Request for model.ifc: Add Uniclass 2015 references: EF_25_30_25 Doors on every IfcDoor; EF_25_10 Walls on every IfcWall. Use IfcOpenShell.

First a look at what the model holds.

```python
import ifcopenshell

model = ifcopenshell.open("model.ifc")
print(model.schema)
print("classifications:", [c.Name for c in model.by_type("IfcClassification")])
for ifc_class in ("IfcDoor", "IfcRoof", "IfcStair", "IfcWall", "IfcWindow"):
    print(ifc_class, len(model.by_type(ifc_class)))
```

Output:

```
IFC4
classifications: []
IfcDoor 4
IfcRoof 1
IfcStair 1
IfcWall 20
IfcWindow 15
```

```python
import ifcopenshell
import ifcopenshell.api.classification

model = ifcopenshell.open("model.ifc")

system = ifcopenshell.api.classification.add_classification(model, classification="Uniclass 2015")

codes = {
    "IfcDoor": ("EF_25_30_25", "Doors"),
    "IfcWall": ("EF_25_10", "Walls"),
}
for ifc_class, (code, name) in codes.items():
    products = model.by_type(ifc_class)
    ifcopenshell.api.classification.add_reference(
        model, products=products, classification=system, identification=code, name=name
    )
    print(code, len(products))

model.write("model-out.ifc")
```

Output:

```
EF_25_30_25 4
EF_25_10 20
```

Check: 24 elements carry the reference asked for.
